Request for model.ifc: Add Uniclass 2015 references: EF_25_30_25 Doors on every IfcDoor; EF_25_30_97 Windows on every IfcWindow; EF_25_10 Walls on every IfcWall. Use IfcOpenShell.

First a look at what the model holds.

```python
import ifcopenshell

model = ifcopenshell.open("model.ifc")
print(model.schema)
print("classifications:", [c.Name for c in model.by_type("IfcClassification")])
for ifc_class in ("IfcDoor", "IfcRoof", "IfcStair", "IfcWall", "IfcWindow"):
    print(ifc_class, len(model.by_type(ifc_class)))
```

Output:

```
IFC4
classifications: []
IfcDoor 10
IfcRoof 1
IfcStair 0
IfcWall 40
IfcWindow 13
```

```python
import ifcopenshell
import ifcopenshell.api.classification

model = ifcopenshell.open("model.ifc")

system = ifcopenshell.api.classification.add_classification(model, classification="Uniclass 2015")

codes = {
    "IfcDoor": ("EF_25_30_25", "Doors"),
    "IfcWindow": ("EF_25_30_97", "Windows"),
    "IfcWall": ("EF_25_10", "Walls"),
}
for ifc_class, (code, name) in codes.items():
    products = model.by_type(ifc_class)
    ifcopenshell.api.classification.add_reference(
        model, products=products, classification=system, identification=code, name=name
    )
    print(code, len(products))

model.write("model_updated.ifc")
```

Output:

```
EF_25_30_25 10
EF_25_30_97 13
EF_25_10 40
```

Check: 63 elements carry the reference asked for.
